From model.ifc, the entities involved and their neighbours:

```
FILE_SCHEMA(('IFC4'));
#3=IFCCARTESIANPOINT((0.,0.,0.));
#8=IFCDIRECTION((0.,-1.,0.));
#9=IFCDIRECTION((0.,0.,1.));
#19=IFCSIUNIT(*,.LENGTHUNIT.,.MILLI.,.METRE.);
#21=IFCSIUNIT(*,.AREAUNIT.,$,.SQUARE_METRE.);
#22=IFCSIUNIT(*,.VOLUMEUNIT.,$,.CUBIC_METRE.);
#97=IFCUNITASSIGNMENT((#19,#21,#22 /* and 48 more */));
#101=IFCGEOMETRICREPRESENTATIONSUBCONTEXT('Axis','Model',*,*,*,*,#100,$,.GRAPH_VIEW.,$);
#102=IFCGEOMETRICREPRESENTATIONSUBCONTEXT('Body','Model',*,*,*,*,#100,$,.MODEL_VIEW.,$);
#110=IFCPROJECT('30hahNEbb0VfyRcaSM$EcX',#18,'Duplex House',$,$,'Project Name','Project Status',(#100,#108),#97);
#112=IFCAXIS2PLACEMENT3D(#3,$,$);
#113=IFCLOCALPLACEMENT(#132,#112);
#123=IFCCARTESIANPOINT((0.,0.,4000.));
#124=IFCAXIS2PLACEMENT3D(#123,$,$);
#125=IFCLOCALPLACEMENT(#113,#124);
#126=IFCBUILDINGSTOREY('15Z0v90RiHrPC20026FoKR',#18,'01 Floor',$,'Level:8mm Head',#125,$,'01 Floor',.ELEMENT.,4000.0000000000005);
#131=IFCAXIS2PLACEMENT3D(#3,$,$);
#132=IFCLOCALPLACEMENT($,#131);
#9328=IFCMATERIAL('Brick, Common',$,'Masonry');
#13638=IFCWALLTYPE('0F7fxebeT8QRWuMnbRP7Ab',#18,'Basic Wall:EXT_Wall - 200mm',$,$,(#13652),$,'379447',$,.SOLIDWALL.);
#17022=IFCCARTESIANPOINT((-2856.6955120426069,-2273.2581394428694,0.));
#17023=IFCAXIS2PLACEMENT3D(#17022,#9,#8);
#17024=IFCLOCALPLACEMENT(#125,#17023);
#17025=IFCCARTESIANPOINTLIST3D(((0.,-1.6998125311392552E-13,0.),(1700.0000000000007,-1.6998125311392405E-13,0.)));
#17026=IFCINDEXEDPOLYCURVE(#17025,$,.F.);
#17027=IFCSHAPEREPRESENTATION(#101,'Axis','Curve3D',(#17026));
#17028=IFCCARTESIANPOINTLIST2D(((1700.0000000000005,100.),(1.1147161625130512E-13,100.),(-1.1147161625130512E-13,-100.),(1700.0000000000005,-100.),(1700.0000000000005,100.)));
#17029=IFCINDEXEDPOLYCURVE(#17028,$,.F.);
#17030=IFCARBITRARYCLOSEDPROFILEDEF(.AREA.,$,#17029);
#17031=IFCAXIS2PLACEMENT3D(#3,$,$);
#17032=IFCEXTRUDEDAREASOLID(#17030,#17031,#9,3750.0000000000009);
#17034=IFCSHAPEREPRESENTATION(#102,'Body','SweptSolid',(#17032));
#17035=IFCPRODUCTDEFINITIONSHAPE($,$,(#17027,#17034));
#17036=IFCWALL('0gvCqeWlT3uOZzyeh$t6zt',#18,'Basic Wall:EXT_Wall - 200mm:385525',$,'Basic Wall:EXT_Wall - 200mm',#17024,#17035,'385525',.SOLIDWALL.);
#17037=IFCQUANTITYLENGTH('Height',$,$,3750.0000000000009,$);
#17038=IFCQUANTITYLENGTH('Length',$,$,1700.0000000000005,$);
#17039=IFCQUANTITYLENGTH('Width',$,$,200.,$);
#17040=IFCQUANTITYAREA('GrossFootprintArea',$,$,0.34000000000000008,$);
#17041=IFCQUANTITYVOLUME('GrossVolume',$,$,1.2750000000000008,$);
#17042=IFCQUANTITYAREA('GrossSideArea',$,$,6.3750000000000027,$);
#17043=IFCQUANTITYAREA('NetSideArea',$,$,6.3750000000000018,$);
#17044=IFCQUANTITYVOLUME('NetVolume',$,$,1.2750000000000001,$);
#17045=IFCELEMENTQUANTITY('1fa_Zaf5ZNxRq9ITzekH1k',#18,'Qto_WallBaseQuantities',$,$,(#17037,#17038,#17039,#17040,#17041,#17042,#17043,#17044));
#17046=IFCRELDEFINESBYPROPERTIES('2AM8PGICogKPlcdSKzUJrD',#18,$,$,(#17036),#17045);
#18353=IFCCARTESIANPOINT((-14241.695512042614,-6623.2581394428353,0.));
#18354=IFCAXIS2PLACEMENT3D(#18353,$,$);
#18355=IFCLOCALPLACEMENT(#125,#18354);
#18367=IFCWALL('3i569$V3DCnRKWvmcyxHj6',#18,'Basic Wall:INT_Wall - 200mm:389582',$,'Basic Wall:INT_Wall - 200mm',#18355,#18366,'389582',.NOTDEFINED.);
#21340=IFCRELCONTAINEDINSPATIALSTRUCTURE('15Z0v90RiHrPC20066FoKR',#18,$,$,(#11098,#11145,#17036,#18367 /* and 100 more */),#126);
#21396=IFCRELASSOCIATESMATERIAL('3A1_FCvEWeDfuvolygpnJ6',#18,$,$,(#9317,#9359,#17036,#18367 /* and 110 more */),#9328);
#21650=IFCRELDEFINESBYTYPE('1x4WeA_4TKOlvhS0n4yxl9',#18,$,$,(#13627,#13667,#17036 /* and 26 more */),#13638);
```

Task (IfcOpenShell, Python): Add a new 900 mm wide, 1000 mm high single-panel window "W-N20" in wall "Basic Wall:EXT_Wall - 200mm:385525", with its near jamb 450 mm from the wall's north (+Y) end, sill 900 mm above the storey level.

```python
import numpy as np
import ifcopenshell
import ifcopenshell.api.feature
import ifcopenshell.api.geometry
import ifcopenshell.api.pset
import ifcopenshell.api.root
import ifcopenshell.api.spatial
import ifcopenshell.geom
import ifcopenshell.util.element
import ifcopenshell.util.placement
import ifcopenshell.util.representation
import ifcopenshell.util.shape
import ifcopenshell.util.unit

model = ifcopenshell.open("model.ifc")
unit_scale = ifcopenshell.util.unit.calculate_unit_scale(model)
area_scale = ifcopenshell.util.unit.calculate_unit_scale(model, "AREAUNIT")
volume_scale = ifcopenshell.util.unit.calculate_unit_scale(model, "VOLUMEUNIT")
settings = ifcopenshell.geom.settings()


def volume(element):
    """Net volume in cubic metres, openings subtracted."""
    shape = ifcopenshell.geom.create_shape(settings, element)
    return ifcopenshell.util.shape.get_volume(shape.geometry)


wall = model.by_guid("0gvCqeWlT3uOZzyeh$t6zt")
storey = ifcopenshell.util.element.get_container(wall, ifc_class="IfcBuildingStorey")
context = ifcopenshell.util.representation.get_context(model, "Model", "Body", "MODEL_VIEW")
before = volume(wall)

width, height, from_end, sill = 0.9, 1, 0.45, 0.9  # metres

# The wall runs along its own X axis, and the end named is its -X end.
wall_shape = ifcopenshell.geom.create_shape(settings, wall)
x, y, z = ifcopenshell.util.shape.get_vertices(wall_shape.geometry).T
start = x.min() + from_end
face, thickness = float(y.min()), float(y.max() - y.min())
wall_matrix = ifcopenshell.util.placement.get_local_placement(wall.ObjectPlacement)
level = ifcopenshell.util.placement.get_local_placement(storey.ObjectPlacement)[2, 3]


def in_wall(x, y):
    """Placement at x, y metres in the wall's axes, at sill height."""
    matrix = wall_matrix.copy()
    matrix[:, 3] = wall_matrix @ np.array([x / unit_scale, y / unit_scale, 0.0, 1.0])
    matrix[2, 3] = level + sill / unit_scale
    return matrix


# Opening: a box that overshoots both wall faces by 50 mm.
opening = ifcopenshell.api.root.create_entity(model, ifc_class="IfcOpeningElement", predefined_type="OPENING")
box = ifcopenshell.api.geometry.add_wall_representation(
    model, context=context, length=width, height=height, thickness=thickness + 0.1
)
ifcopenshell.api.geometry.assign_representation(model, product=opening, representation=box)
ifcopenshell.api.geometry.edit_object_placement(model, product=opening, matrix=in_wall(start, face - 0.05), is_si=False)
ifcopenshell.api.feature.add_feature(model, feature=opening, element=wall)

window = ifcopenshell.api.root.create_entity(model, ifc_class="IfcWindow", name="W-N20", predefined_type="WINDOW")
window.OverallWidth, window.OverallHeight = width / unit_scale, height / unit_scale
window.PartitioningType = "SINGLE_PANEL"
body = ifcopenshell.api.geometry.add_window_representation(
    model,
    context=context,
    overall_width=window.OverallWidth,
    overall_height=window.OverallHeight,
    partition_type="SINGLE_PANEL",
)
ifcopenshell.api.geometry.assign_representation(model, product=window, representation=body)
ifcopenshell.api.spatial.assign_container(model, products=[window], relating_structure=storey)
ifcopenshell.api.feature.add_filling(model, opening=opening, element=window)

# Centre the window in the wall's thickness.
ifcopenshell.api.geometry.edit_object_placement(model, product=window, matrix=in_wall(start, face), is_si=False)
window_shape = ifcopenshell.geom.create_shape(settings, window)
depth = ifcopenshell.util.shape.get_vertices(window_shape.geometry)[:, 1]
offset = face + thickness / 2 - (depth.min() + depth.max()) / 2
ifcopenshell.api.geometry.edit_object_placement(model, product=window, matrix=in_wall(start, offset), is_si=False)

after = volume(wall)

# Update the wall's stored quantities.
qto = model.by_id(ifcopenshell.util.element.get_pset(wall, "Qto_WallBaseQuantities", should_inherit=False)["id"])
ifcopenshell.api.pset.edit_qto(model, qto=qto, properties={
    "NetSideArea": after / thickness / area_scale,
    "NetVolume": after / volume_scale,
})

print(f"wall volume {before:.3f} -> {after:.3f} m3")

model.write("model_rev.ifc")
```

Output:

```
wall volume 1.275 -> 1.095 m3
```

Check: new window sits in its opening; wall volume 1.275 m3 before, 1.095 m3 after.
